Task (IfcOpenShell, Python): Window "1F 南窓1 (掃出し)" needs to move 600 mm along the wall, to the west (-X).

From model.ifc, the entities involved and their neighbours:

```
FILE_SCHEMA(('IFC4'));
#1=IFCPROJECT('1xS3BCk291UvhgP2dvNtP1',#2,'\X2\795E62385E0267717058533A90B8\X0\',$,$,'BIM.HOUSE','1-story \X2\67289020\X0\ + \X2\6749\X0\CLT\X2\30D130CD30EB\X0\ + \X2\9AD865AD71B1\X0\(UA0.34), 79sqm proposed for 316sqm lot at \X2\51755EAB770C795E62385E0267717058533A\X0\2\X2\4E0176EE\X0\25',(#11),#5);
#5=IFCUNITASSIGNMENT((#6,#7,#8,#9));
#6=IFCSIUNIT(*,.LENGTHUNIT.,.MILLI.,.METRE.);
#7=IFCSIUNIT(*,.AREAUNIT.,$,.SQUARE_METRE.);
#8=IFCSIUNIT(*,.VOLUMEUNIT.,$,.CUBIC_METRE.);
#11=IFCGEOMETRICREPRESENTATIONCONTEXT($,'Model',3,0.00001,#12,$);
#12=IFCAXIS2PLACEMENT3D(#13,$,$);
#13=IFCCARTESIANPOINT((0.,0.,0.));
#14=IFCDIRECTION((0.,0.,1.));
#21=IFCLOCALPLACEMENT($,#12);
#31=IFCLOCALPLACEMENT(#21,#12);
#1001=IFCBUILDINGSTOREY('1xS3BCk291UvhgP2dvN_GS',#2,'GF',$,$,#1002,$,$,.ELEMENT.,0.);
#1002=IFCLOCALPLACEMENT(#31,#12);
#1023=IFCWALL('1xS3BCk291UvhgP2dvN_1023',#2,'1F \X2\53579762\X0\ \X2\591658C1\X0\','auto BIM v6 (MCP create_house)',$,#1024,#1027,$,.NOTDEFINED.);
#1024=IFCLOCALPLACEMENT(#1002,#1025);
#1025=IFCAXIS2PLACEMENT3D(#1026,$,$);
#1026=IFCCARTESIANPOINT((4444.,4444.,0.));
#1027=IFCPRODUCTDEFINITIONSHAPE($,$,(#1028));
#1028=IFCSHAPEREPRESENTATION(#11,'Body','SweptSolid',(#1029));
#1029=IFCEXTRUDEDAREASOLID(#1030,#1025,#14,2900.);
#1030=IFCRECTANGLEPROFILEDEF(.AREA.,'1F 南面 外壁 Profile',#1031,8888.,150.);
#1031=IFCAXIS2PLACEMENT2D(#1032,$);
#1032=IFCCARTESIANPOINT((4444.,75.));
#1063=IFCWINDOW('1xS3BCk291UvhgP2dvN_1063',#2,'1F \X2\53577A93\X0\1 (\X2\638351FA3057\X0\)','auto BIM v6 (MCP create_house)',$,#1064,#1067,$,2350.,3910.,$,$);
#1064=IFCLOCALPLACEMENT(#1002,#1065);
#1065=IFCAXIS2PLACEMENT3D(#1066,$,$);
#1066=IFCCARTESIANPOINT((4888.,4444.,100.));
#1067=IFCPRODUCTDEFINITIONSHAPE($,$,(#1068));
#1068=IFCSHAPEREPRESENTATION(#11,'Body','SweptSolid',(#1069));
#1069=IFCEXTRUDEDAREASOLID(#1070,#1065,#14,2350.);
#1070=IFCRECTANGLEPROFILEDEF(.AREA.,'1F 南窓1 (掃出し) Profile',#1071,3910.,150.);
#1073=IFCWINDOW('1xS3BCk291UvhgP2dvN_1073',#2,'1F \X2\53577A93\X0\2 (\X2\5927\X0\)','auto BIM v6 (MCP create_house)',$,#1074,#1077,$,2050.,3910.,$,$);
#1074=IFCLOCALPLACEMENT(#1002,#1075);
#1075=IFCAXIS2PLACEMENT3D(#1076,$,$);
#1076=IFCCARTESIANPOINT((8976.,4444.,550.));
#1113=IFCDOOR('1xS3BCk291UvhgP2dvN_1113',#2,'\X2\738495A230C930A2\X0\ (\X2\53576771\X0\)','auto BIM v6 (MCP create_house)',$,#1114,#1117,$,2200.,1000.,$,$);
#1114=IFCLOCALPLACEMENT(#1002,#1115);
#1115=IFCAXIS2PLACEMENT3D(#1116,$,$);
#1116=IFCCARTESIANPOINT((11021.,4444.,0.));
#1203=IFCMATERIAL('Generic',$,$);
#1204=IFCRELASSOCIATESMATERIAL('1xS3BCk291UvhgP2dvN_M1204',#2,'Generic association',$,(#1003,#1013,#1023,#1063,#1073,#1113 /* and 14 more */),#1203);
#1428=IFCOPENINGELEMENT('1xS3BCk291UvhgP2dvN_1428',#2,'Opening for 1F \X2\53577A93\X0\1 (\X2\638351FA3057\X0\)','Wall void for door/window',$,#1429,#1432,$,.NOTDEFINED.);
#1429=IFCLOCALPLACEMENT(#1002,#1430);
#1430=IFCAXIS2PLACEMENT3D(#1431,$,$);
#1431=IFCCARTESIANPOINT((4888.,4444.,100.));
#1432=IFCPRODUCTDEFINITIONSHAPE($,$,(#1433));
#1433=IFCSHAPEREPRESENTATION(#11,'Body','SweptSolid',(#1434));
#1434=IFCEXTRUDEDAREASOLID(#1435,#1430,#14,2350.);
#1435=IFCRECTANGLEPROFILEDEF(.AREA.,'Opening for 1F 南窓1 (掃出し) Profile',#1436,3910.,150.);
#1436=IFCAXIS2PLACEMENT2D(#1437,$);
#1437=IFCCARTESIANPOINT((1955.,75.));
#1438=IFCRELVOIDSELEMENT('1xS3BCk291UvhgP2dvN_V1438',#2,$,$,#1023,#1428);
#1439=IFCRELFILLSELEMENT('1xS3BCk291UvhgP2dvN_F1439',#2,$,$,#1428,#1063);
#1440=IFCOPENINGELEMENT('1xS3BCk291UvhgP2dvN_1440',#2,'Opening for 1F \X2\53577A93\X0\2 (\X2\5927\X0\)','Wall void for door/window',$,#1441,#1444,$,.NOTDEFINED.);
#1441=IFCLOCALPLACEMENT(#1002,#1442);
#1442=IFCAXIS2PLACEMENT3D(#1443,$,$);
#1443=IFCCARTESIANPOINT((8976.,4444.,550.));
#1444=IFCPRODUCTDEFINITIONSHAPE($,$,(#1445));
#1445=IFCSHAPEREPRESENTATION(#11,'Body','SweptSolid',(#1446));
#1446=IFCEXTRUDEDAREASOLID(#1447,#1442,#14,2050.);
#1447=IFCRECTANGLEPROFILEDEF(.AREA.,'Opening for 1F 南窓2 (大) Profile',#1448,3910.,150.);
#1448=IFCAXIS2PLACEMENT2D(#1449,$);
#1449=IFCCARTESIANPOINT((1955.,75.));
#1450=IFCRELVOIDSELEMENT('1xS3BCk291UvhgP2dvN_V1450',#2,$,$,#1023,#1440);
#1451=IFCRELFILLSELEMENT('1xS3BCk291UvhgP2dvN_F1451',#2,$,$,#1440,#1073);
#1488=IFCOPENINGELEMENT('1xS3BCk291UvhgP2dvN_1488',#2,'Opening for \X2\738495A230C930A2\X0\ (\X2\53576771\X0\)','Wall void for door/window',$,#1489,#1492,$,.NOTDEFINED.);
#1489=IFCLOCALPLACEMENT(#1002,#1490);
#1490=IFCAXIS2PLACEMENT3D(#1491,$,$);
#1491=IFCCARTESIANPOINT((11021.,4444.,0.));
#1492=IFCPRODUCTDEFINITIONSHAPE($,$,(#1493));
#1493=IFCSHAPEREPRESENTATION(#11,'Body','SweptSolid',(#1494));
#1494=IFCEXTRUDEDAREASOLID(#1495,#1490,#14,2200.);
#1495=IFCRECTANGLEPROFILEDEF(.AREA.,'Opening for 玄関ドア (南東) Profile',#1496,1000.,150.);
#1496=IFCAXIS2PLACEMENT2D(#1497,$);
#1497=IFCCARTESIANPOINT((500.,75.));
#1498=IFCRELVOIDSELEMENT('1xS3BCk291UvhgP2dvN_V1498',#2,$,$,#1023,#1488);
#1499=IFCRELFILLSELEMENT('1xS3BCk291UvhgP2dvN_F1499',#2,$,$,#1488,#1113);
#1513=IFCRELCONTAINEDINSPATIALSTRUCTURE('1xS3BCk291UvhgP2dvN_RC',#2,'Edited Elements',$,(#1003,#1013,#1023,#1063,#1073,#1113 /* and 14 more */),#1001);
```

```python
import ifcopenshell
import ifcopenshell.api.geometry
import ifcopenshell.util.placement

model = ifcopenshell.open("model.ifc")

window = model.by_guid("1xS3BCk291UvhgP2dvN_1063")
opening = window.FillsVoids[0].RelatingOpeningElement
wall = opening.VoidsElements[0].RelatingBuildingElement

wall_matrix = ifcopenshell.util.placement.get_local_placement(wall.ObjectPlacement)
shift = wall_matrix[:3, 0] * -600.0
before = ifcopenshell.util.placement.get_local_placement(window.ObjectPlacement)[:3, 3].copy()

# The window is not placed relative to its opening, so move both.
for product in (opening, window):
    matrix = ifcopenshell.util.placement.get_local_placement(product.ObjectPlacement)
    matrix[:3, 3] += shift
    ifcopenshell.api.geometry.edit_object_placement(model, product=product, matrix=matrix, is_si=False)

after = ifcopenshell.util.placement.get_local_placement(window.ObjectPlacement)[:3, 3]
print("window moved by", (after - before).round(3) + 0.0)

model.write("model_rev.ifc")
```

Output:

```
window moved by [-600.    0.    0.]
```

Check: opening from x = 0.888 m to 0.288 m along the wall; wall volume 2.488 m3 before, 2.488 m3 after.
